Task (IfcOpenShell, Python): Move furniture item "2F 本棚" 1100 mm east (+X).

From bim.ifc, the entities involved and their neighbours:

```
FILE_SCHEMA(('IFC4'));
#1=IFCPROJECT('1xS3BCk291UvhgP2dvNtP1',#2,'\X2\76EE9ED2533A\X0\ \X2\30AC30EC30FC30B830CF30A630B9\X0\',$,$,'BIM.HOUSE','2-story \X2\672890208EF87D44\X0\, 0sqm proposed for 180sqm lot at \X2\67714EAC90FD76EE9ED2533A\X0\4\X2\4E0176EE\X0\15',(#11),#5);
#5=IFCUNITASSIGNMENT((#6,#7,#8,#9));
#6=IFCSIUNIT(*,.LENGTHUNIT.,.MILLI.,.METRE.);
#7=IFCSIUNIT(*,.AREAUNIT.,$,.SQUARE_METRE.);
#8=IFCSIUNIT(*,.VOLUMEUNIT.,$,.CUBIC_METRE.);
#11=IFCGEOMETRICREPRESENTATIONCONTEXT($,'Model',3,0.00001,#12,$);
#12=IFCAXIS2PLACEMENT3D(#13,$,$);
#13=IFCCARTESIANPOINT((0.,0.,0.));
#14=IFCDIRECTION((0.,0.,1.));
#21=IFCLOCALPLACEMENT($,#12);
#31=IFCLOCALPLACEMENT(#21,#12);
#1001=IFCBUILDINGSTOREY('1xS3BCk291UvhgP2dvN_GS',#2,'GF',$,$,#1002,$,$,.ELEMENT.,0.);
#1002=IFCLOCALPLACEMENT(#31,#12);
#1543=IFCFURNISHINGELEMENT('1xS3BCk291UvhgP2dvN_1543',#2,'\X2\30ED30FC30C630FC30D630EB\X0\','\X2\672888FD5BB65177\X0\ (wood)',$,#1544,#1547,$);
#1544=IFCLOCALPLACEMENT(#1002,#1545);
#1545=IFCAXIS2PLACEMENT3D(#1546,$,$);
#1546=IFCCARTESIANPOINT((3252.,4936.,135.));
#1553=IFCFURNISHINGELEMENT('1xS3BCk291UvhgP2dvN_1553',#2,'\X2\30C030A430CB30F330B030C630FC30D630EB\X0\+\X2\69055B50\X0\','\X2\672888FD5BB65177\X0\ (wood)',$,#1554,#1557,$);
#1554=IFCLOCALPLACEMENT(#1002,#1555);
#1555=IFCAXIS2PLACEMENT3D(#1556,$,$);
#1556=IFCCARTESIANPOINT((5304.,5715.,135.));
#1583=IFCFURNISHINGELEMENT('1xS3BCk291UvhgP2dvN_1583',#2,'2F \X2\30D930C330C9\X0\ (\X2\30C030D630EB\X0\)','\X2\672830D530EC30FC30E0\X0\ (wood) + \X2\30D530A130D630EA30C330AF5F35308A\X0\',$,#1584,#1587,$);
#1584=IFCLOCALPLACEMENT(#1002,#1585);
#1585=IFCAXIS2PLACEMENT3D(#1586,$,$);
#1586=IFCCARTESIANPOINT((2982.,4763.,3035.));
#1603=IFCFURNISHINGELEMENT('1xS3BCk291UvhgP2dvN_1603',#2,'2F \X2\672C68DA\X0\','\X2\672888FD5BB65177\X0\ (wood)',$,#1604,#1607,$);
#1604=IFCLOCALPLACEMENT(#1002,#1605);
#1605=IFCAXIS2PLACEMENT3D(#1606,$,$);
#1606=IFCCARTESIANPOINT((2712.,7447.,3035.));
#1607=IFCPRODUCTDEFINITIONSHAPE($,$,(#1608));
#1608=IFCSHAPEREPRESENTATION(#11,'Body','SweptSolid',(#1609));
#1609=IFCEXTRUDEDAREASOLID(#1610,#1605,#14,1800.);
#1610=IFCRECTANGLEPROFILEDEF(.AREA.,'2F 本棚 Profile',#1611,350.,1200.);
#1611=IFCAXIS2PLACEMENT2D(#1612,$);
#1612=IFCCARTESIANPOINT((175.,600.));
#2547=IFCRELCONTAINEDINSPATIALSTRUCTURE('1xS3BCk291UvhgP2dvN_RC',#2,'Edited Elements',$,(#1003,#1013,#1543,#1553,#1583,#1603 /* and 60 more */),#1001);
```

```python
import ifcopenshell
import ifcopenshell.api.geometry
import ifcopenshell.util.placement

model = ifcopenshell.open("bim.ifc")

item = model.by_guid("1xS3BCk291UvhgP2dvN_1603")
matrix = ifcopenshell.util.placement.get_local_placement(item.ObjectPlacement)
matrix[0, 3] += 1100.0
ifcopenshell.api.geometry.edit_object_placement(model, product=item, matrix=matrix, is_si=False)

print(ifcopenshell.util.placement.get_local_placement(item.ObjectPlacement).round(3) + 0.0)

model.write("bim_edited.ifc")
```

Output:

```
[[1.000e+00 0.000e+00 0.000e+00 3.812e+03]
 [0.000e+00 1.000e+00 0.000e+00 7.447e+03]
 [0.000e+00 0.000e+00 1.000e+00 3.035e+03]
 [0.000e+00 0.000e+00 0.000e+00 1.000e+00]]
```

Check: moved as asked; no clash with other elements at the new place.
